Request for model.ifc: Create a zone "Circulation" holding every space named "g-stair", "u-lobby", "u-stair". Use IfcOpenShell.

First a look at what the model holds.

```python
import ifcopenshell

model = ifcopenshell.open("model.ifc")
print(model.schema)
seen = {}
for space in model.by_type("IfcSpace"):
    seen[space.LongName] = seen.get(space.LongName, 0) + 1
for name, count in sorted(seen.items(), key=str):
    print(count, "x", name)
print("zones:", [z.Name for z in model.by_type("IfcZone")][:20])
```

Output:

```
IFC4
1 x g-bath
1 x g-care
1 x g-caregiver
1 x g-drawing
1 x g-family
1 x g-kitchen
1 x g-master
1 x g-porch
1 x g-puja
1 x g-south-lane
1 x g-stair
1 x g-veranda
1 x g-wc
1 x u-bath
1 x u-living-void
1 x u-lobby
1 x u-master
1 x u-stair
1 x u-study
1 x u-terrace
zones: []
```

```python
import ifcopenshell
import ifcopenshell.api.group
import ifcopenshell.api.root

model = ifcopenshell.open("model.ifc")

names = {"g-stair", "u-lobby", "u-stair"}
spaces = [s for s in model.by_type("IfcSpace") if s.LongName in names]

zone = ifcopenshell.api.root.create_entity(model, ifc_class="IfcZone", name="Circulation")
ifcopenshell.api.group.assign_group(model, products=spaces, group=zone)
print(len(spaces), "spaces in", zone.Name)

model.write("model_updated.ifc")
```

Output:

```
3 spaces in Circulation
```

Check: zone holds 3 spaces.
